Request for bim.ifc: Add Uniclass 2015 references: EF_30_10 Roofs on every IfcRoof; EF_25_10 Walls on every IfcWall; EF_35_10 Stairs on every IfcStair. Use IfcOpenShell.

First a look at what the model holds.

```python
import ifcopenshell

model = ifcopenshell.open("bim.ifc")
print(model.schema)
print("classifications:", [c.Name for c in model.by_type("IfcClassification")])
for ifc_class in ("IfcDoor", "IfcRoof", "IfcStair", "IfcWall", "IfcWindow"):
    print(ifc_class, len(model.by_type(ifc_class)))
```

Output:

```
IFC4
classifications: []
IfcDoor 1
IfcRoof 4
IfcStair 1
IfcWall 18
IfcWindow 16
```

```python
import ifcopenshell
import ifcopenshell.api.classification

model = ifcopenshell.open("bim.ifc")

system = ifcopenshell.api.classification.add_classification(model, classification="Uniclass 2015")

codes = {
    "IfcRoof": ("EF_30_10", "Roofs"),
    "IfcWall": ("EF_25_10", "Walls"),
    "IfcStair": ("EF_35_10", "Stairs"),
}
for ifc_class, (code, name) in codes.items():
    products = model.by_type(ifc_class)
    ifcopenshell.api.classification.add_reference(
        model, products=products, classification=system, identification=code, name=name
    )
    print(code, len(products))

model.write("bim_updated.ifc")
```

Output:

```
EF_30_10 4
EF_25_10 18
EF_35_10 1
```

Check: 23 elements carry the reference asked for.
